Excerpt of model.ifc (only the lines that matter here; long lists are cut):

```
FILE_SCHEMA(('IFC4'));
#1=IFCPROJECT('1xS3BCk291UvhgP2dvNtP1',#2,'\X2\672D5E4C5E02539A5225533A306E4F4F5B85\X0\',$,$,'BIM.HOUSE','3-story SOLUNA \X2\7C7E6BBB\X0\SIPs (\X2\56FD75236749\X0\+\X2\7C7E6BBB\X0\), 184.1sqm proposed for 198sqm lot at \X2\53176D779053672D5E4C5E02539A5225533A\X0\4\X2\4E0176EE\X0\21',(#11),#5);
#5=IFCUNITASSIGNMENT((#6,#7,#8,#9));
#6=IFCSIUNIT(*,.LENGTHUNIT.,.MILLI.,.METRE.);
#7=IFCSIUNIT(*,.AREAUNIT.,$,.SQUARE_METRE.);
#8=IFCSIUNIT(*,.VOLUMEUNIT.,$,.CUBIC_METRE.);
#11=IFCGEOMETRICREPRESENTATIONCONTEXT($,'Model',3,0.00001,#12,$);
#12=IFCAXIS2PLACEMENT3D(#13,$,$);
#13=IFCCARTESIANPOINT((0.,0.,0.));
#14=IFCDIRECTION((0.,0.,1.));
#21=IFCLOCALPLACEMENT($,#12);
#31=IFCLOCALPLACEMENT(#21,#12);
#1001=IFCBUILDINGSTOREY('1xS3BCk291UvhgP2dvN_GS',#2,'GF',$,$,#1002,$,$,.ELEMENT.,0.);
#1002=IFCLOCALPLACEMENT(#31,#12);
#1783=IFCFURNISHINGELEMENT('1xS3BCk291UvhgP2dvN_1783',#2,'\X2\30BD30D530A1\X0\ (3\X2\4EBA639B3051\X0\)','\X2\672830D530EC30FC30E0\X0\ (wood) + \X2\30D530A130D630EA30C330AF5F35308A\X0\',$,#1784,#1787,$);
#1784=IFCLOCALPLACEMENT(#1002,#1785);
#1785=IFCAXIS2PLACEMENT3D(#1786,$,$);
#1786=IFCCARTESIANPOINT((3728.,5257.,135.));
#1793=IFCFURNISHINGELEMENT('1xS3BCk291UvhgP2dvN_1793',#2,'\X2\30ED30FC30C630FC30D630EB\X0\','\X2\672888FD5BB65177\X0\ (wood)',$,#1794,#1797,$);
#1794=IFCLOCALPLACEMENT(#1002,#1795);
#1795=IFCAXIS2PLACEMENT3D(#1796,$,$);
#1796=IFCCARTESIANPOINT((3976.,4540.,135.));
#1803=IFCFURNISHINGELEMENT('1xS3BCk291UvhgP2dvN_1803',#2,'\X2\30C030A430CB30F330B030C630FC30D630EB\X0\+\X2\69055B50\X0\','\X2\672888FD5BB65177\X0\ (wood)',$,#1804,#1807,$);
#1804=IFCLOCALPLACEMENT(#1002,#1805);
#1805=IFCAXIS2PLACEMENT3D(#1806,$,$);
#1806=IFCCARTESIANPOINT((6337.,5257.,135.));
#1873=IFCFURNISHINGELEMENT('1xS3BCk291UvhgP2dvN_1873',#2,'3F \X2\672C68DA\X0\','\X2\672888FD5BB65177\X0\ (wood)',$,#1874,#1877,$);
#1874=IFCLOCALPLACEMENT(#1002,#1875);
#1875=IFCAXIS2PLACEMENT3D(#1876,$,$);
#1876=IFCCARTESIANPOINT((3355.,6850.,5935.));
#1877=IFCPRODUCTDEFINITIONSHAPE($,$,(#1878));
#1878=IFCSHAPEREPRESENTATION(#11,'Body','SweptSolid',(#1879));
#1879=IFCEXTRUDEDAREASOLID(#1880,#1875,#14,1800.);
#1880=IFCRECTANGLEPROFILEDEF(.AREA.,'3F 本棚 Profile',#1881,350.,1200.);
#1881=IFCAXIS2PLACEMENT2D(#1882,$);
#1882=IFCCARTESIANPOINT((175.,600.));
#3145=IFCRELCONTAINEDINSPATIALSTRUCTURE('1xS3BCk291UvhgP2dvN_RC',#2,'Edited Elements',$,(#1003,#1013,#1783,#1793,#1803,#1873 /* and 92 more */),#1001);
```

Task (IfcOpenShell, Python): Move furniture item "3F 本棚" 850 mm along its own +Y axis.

```python
import ifcopenshell
import ifcopenshell.api.geometry
import ifcopenshell.util.placement

model = ifcopenshell.open("model.ifc")

item = model.by_id(1873)
matrix = ifcopenshell.util.placement.get_local_placement(item.ObjectPlacement)
matrix[:3, 3] += matrix[:3, 1] * 850.0
ifcopenshell.api.geometry.edit_object_placement(model, product=item, matrix=matrix, is_si=False)

print(ifcopenshell.util.placement.get_local_placement(item.ObjectPlacement).round(3) + 0.0)

model.write("model_rev.ifc")
```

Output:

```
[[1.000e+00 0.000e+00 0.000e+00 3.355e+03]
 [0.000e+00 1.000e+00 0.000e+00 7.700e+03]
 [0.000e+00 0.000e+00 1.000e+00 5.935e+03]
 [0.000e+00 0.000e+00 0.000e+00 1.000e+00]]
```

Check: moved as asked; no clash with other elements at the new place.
